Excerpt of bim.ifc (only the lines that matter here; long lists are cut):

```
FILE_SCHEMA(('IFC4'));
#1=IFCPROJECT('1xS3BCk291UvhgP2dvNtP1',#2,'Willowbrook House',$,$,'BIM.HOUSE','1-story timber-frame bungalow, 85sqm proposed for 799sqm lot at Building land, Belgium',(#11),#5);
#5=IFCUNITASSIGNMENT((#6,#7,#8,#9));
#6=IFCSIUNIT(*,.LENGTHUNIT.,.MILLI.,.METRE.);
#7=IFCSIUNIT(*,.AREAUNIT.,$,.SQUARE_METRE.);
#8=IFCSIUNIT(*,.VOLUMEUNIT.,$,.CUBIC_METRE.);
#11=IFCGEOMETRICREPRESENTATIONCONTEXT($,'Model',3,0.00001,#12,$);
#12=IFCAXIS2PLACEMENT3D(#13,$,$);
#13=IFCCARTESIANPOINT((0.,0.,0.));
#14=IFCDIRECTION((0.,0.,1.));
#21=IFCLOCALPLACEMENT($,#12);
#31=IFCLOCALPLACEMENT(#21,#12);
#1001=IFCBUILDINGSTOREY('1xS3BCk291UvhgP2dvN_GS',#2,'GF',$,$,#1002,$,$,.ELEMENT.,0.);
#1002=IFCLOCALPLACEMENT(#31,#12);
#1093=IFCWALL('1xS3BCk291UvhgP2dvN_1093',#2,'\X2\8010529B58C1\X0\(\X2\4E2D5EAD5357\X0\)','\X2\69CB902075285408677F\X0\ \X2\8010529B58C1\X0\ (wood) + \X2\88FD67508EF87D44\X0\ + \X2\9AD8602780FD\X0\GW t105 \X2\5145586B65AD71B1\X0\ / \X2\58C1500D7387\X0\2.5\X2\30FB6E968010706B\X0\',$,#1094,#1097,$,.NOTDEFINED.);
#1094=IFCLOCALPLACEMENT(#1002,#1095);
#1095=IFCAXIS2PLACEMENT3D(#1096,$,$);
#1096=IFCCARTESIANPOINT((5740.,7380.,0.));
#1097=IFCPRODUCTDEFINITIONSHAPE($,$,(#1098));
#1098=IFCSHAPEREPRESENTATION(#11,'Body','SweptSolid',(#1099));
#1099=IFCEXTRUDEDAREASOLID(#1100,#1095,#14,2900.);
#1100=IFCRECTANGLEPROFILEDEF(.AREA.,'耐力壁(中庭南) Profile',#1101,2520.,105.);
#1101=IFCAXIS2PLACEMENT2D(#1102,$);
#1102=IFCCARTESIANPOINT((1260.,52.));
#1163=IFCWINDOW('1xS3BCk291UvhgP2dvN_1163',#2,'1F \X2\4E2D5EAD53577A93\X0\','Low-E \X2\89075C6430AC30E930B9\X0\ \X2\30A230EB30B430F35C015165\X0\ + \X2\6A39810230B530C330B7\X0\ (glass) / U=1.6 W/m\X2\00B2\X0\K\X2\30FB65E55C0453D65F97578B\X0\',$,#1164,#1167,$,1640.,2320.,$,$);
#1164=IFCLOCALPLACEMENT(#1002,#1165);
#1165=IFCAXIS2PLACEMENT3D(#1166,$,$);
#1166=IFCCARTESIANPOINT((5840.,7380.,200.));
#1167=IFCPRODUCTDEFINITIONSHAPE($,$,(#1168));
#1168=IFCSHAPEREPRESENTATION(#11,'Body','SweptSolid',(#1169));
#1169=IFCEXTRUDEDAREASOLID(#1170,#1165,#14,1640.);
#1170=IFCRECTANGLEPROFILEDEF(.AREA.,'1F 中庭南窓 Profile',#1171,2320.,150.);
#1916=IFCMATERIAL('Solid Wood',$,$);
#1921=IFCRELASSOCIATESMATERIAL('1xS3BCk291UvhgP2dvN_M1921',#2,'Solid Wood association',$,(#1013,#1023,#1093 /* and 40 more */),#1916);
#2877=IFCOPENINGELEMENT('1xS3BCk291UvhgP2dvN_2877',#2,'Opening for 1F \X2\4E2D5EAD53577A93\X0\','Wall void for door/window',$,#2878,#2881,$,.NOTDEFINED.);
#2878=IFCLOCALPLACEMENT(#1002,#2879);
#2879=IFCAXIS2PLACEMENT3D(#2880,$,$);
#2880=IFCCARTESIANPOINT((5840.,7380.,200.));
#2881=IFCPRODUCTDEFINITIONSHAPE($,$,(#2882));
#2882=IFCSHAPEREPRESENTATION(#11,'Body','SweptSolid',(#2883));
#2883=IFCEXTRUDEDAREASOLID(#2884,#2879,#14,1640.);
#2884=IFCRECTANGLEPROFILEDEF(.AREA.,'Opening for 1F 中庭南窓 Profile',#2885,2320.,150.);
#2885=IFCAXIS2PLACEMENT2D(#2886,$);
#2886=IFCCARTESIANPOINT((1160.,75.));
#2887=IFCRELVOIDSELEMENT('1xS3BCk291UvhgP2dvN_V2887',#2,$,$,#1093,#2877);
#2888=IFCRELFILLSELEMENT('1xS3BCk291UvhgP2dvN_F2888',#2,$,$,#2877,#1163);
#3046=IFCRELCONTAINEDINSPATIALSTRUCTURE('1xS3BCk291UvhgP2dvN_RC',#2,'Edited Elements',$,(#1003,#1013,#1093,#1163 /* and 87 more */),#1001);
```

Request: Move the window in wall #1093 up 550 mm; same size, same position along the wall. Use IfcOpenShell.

```python
import numpy as np
import ifcopenshell
import ifcopenshell.api.geometry
import ifcopenshell.util.placement
import ifcopenshell.util.unit

model = ifcopenshell.open("bim.ifc")
unit_scale = ifcopenshell.util.unit.calculate_unit_scale(model)

window = model.by_guid("1xS3BCk291UvhgP2dvN_1163")
opening = window.FillsVoids[0].RelatingOpeningElement
dz = 0.55 / unit_scale

shift = np.array([0.0, 0.0, dz])
# The window is not placed relative to its opening, so move both.
for product in (opening, window):
    matrix = ifcopenshell.util.placement.get_local_placement(product.ObjectPlacement)
    matrix[:3, 3] += shift
    ifcopenshell.api.geometry.edit_object_placement(model, product=product, matrix=matrix, is_si=False)

print(f"moved by {dz * unit_scale:+.3f} m")

model.write("bim-out.ifc")
```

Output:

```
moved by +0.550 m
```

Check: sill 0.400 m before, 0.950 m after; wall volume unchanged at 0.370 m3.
